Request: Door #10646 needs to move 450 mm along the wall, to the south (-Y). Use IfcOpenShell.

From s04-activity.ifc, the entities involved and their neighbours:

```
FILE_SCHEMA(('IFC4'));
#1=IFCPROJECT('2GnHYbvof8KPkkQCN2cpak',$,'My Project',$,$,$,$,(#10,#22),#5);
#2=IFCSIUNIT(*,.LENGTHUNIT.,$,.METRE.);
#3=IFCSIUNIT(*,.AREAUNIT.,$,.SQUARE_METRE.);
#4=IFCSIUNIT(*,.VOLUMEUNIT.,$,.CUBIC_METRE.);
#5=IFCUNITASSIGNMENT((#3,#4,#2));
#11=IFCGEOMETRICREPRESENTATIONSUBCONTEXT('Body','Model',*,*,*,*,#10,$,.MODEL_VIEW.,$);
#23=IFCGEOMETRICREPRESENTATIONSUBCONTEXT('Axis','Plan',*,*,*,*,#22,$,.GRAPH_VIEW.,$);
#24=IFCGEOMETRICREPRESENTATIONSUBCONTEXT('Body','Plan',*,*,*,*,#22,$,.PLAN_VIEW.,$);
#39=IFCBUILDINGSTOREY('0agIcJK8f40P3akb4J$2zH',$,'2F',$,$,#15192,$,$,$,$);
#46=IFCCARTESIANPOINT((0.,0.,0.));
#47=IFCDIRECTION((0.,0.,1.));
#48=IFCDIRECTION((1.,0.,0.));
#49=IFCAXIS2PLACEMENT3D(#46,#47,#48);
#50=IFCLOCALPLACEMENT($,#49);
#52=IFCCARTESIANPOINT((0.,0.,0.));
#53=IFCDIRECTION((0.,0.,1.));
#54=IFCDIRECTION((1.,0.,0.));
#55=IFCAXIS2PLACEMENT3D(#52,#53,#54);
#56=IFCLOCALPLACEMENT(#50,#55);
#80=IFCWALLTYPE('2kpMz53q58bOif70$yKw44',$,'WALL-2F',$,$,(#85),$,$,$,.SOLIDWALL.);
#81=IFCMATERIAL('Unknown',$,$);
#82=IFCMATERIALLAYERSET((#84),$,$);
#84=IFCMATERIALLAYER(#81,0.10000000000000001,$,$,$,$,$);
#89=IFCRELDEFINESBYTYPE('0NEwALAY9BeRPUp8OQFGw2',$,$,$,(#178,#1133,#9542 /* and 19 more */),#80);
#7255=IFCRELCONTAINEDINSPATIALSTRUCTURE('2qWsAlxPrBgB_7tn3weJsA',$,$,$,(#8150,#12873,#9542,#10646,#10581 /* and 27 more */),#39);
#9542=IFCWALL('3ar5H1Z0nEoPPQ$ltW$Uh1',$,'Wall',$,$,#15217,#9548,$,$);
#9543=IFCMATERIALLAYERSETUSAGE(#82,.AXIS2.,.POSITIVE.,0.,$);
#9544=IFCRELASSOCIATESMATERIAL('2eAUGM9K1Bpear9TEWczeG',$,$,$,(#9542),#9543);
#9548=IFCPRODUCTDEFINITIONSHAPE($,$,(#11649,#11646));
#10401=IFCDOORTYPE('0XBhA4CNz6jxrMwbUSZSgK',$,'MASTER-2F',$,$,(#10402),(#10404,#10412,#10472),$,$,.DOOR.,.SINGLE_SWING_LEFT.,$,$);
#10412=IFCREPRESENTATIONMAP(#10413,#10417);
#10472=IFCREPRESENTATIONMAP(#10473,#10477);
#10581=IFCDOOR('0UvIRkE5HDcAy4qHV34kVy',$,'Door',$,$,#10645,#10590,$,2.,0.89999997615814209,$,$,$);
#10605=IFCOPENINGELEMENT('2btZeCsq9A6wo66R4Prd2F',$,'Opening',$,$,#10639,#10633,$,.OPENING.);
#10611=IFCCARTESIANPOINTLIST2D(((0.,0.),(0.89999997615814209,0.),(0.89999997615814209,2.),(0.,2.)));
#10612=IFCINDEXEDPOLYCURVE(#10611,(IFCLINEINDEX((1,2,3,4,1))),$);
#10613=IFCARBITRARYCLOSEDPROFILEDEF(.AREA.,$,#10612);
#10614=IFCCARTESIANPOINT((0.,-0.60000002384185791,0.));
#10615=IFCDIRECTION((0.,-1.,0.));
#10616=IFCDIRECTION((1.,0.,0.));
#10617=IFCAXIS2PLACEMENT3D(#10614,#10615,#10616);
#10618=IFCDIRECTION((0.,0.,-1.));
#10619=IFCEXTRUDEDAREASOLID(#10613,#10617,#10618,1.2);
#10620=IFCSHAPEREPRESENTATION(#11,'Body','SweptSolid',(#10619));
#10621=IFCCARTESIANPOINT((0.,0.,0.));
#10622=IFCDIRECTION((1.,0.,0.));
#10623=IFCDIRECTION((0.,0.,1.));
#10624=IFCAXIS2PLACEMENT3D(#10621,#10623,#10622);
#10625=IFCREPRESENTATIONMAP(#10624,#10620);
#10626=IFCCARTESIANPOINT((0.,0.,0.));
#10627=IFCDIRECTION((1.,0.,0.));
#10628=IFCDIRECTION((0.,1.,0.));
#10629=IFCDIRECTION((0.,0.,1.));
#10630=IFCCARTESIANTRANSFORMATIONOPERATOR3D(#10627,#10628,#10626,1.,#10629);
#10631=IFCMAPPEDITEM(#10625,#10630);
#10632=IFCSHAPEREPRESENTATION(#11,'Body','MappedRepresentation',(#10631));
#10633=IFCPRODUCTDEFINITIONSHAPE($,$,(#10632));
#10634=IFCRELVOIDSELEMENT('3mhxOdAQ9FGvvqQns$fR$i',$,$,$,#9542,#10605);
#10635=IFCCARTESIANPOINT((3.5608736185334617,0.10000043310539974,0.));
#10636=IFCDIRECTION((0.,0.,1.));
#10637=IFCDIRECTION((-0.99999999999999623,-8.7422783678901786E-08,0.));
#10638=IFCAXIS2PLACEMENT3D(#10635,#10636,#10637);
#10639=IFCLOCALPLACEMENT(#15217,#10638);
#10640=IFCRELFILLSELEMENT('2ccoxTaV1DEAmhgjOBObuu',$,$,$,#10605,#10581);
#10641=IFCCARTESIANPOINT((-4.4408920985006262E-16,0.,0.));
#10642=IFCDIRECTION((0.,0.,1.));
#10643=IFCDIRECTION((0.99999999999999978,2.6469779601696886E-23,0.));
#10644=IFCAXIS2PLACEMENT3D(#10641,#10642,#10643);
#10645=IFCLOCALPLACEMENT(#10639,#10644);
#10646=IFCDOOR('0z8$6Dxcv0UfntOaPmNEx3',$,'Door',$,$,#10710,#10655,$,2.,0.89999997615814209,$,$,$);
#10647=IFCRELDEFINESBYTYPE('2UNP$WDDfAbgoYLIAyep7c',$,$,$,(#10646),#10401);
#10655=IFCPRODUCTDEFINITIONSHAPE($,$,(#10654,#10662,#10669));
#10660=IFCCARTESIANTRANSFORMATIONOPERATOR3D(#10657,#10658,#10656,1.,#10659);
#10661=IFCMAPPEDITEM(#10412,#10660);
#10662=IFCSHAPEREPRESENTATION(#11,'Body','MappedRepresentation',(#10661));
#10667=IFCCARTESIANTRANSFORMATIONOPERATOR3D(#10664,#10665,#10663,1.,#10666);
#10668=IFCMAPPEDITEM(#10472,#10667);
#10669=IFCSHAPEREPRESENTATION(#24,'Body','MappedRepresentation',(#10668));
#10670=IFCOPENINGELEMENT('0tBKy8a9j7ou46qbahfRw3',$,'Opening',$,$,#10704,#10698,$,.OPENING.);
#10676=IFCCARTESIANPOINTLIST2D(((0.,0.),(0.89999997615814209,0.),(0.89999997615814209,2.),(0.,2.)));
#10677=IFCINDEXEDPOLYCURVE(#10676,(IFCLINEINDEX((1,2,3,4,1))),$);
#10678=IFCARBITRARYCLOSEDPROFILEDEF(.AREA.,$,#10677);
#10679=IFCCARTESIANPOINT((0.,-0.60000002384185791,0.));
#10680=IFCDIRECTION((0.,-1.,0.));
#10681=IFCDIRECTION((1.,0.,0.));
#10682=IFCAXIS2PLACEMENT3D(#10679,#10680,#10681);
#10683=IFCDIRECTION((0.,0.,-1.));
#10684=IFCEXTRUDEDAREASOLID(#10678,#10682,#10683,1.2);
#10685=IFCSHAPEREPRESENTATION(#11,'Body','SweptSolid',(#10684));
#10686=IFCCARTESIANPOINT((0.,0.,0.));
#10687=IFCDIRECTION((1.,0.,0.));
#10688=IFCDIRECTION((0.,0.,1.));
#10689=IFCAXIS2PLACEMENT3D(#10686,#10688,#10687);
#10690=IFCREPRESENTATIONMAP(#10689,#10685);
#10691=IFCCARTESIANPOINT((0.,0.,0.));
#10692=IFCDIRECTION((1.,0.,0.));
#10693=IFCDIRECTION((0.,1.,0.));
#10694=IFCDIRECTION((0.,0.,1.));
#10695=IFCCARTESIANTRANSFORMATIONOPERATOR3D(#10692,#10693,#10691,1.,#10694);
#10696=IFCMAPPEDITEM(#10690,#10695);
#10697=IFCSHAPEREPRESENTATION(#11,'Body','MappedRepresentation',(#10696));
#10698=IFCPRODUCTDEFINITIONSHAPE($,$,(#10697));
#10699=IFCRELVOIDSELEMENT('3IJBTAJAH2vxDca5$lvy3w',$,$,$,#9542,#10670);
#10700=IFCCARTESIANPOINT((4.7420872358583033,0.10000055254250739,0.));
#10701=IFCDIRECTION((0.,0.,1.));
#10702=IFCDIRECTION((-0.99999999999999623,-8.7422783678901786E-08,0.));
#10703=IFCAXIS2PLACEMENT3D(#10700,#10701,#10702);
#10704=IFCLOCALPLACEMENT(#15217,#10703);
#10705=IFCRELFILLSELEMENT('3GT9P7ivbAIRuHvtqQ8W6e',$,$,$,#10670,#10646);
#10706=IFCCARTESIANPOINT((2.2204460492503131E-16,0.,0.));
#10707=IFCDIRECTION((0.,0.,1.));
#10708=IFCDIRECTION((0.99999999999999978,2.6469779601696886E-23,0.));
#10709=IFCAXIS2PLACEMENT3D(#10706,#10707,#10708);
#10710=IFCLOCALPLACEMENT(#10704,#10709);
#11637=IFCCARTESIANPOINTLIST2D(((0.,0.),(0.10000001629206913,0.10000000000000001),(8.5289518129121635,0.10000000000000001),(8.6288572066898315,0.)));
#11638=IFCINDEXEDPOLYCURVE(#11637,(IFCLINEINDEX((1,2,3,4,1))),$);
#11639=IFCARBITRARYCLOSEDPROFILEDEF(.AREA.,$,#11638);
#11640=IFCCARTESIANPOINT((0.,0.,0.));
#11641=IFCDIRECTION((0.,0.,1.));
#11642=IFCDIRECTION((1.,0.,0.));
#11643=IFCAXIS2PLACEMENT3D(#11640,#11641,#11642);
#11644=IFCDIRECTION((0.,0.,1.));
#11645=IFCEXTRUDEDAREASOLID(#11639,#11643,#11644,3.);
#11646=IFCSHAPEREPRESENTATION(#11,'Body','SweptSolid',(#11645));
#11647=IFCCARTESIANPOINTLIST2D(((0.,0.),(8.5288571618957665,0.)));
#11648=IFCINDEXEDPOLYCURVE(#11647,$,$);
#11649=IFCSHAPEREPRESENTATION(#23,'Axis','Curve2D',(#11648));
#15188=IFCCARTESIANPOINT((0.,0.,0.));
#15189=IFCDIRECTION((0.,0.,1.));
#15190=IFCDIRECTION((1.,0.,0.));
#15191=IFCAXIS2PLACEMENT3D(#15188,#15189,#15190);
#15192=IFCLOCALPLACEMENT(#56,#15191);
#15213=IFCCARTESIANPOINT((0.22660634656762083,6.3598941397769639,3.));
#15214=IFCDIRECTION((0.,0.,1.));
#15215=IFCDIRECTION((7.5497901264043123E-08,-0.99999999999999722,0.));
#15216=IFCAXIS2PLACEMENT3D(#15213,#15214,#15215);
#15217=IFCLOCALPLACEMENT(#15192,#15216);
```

```python
import ifcopenshell
import ifcopenshell.api.geometry
import ifcopenshell.util.placement

model = ifcopenshell.open("s04-activity.ifc")

door = model.by_guid("0z8$6Dxcv0UfntOaPmNEx3")
opening = door.FillsVoids[0].RelatingOpeningElement
wall = opening.VoidsElements[0].RelatingBuildingElement

wall_matrix = ifcopenshell.util.placement.get_local_placement(wall.ObjectPlacement)
shift = wall_matrix[:3, 0] * 0.45
before = ifcopenshell.util.placement.get_local_placement(door.ObjectPlacement)[:3, 3].copy()

# The door is placed relative to its opening, so it follows when the opening moves.
matrix = ifcopenshell.util.placement.get_local_placement(opening.ObjectPlacement)
matrix[:3, 3] += shift
ifcopenshell.api.geometry.edit_object_placement(
    model, product=opening, matrix=matrix, is_si=False, should_transform_children=True
)

after = ifcopenshell.util.placement.get_local_placement(door.ObjectPlacement)[:3, 3]
print("door moved by", (after - before).round(3) + 0.0)

model.write("s04-activity_rev.ifc")
```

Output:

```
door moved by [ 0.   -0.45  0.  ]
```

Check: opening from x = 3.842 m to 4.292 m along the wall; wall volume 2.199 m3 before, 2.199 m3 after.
